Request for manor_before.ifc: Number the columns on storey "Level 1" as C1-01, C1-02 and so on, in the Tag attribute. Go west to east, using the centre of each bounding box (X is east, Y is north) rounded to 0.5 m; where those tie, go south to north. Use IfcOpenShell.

First a look at what the model holds.

```python
import ifcopenshell
import ifcopenshell.util.element
import ifcopenshell.util.placement

model = ifcopenshell.open("manor_before.ifc")
print(model.schema)
storey = next(s for s in model.by_type("IfcBuildingStorey") if s.Name == "Level 1")
columns = [e for e in ifcopenshell.util.element.get_decomposition(storey) if e.is_a("IfcColumn")]
for e in sorted(columns, key=lambda e: e.id()):
    origin = ifcopenshell.util.placement.get_local_placement(e.ObjectPlacement)[:3, 3]
    print(e.id(), e.Tag, e.Name, origin.round(2) + 0.0, sep=" | ")
```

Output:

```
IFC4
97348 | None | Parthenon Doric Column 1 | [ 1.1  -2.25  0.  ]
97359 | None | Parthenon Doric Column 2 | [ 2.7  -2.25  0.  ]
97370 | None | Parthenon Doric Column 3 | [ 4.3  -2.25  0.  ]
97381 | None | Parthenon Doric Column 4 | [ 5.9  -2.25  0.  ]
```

```python
import ifcopenshell
import ifcopenshell.geom
import ifcopenshell.util.element
import ifcopenshell.util.shape

model = ifcopenshell.open("manor_before.ifc")
settings = ifcopenshell.geom.settings()
settings.set("use-world-coords", True)


def centre(element):
    shape = ifcopenshell.geom.create_shape(settings, element)
    return ifcopenshell.util.shape.get_bbox_centroid(shape.geometry)


storey = next(s for s in model.by_type("IfcBuildingStorey") if s.Name == "Level 1")
columns = [e for e in ifcopenshell.util.element.get_decomposition(storey) if e.is_a("IfcColumn")]

# Insertion points can sit at a corner or the storey origin, so sort by the geometry (in metres).
centres = {e: centre(e) for e in columns}
columns.sort(key=lambda e: (round(centres[e][0] / 0.5), centres[e][1]))

for i, e in enumerate(columns, start=1):
    number = f"C1-{i:02d}"
    e.Tag = number
    print(e.id(), number)

model.write("manor_before-out.ifc")
```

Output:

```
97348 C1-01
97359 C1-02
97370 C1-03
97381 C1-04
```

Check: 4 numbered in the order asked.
